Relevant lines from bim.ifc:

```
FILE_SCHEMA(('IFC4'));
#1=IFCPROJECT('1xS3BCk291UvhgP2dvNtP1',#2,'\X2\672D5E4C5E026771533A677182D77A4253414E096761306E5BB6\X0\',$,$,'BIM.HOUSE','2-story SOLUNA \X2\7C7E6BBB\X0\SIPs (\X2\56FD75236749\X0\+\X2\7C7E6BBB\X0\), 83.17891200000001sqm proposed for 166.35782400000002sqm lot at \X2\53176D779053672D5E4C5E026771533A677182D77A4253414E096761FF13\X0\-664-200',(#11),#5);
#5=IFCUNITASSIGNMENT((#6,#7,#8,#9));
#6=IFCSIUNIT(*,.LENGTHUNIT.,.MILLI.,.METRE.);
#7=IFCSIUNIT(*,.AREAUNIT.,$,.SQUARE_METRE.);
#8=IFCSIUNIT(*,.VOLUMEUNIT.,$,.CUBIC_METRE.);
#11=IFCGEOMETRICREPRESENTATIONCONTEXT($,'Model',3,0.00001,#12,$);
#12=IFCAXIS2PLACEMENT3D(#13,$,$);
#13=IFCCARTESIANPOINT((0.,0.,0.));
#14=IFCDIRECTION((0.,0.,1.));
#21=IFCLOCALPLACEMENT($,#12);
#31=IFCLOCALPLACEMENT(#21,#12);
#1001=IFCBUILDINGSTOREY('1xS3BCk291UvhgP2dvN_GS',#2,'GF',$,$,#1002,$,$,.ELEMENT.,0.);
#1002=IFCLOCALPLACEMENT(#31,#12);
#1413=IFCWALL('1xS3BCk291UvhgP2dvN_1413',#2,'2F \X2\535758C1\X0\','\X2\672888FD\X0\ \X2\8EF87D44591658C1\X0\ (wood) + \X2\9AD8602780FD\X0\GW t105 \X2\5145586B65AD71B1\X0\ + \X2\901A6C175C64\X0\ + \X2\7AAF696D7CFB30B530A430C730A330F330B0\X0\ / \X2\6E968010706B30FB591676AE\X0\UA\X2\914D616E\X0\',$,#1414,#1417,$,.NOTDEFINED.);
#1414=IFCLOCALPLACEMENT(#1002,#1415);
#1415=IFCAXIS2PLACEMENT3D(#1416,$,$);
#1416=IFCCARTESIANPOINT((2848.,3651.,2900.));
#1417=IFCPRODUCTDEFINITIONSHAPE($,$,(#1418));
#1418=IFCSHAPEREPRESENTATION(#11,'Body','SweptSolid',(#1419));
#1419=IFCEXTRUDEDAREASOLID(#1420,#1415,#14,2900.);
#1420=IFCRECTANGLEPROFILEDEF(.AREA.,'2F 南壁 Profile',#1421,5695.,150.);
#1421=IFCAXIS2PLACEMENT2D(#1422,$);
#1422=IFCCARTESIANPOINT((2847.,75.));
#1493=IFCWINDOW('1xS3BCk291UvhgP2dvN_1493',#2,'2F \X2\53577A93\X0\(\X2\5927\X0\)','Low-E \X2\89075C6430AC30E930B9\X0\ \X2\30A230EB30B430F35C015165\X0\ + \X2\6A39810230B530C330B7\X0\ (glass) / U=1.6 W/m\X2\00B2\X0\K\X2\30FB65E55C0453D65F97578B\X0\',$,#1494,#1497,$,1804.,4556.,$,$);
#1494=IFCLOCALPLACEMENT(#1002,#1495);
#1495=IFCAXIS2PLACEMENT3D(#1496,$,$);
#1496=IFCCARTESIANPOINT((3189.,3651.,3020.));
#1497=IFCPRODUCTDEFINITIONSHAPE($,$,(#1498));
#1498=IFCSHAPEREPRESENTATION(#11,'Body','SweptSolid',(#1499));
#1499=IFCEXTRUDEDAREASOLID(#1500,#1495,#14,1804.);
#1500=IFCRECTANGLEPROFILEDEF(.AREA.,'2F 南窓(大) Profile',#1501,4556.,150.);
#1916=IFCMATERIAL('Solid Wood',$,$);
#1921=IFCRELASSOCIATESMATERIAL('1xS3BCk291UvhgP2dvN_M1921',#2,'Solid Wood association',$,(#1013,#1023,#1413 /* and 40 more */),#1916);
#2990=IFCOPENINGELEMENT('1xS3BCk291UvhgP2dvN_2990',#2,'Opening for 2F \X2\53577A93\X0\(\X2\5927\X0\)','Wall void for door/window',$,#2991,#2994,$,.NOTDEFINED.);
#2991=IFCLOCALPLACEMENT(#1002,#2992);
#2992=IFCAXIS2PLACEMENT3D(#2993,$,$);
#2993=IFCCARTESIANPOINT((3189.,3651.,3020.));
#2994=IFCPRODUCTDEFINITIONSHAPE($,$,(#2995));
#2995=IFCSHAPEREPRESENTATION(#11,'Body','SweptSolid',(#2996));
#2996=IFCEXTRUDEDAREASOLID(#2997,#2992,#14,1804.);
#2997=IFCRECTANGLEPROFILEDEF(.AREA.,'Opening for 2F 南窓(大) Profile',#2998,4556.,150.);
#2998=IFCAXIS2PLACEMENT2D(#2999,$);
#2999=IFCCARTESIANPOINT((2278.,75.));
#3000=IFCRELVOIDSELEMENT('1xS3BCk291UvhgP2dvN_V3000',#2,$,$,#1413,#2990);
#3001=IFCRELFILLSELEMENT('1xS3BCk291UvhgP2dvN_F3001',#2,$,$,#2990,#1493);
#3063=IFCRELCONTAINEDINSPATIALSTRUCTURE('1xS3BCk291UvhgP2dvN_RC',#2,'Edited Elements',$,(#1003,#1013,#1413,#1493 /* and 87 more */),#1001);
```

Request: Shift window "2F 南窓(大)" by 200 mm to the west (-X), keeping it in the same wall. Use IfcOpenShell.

```python
import ifcopenshell
import ifcopenshell.api.geometry
import ifcopenshell.util.placement

model = ifcopenshell.open("bim.ifc")

window = model.by_guid("1xS3BCk291UvhgP2dvN_1493")
opening = window.FillsVoids[0].RelatingOpeningElement
wall = opening.VoidsElements[0].RelatingBuildingElement

wall_matrix = ifcopenshell.util.placement.get_local_placement(wall.ObjectPlacement)
shift = wall_matrix[:3, 0] * -200.0
before = ifcopenshell.util.placement.get_local_placement(window.ObjectPlacement)[:3, 3].copy()

# The window is not placed relative to its opening, so move both.
for product in (opening, window):
    matrix = ifcopenshell.util.placement.get_local_placement(product.ObjectPlacement)
    matrix[:3, 3] += shift
    ifcopenshell.api.geometry.edit_object_placement(model, product=product, matrix=matrix, is_si=False)

after = ifcopenshell.util.placement.get_local_placement(window.ObjectPlacement)[:3, 3]
print("window moved by", (after - before).round(3) + 0.0)

model.write("bim_v2.ifc")
```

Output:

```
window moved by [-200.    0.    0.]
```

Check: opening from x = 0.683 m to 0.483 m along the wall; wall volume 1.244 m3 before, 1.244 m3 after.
